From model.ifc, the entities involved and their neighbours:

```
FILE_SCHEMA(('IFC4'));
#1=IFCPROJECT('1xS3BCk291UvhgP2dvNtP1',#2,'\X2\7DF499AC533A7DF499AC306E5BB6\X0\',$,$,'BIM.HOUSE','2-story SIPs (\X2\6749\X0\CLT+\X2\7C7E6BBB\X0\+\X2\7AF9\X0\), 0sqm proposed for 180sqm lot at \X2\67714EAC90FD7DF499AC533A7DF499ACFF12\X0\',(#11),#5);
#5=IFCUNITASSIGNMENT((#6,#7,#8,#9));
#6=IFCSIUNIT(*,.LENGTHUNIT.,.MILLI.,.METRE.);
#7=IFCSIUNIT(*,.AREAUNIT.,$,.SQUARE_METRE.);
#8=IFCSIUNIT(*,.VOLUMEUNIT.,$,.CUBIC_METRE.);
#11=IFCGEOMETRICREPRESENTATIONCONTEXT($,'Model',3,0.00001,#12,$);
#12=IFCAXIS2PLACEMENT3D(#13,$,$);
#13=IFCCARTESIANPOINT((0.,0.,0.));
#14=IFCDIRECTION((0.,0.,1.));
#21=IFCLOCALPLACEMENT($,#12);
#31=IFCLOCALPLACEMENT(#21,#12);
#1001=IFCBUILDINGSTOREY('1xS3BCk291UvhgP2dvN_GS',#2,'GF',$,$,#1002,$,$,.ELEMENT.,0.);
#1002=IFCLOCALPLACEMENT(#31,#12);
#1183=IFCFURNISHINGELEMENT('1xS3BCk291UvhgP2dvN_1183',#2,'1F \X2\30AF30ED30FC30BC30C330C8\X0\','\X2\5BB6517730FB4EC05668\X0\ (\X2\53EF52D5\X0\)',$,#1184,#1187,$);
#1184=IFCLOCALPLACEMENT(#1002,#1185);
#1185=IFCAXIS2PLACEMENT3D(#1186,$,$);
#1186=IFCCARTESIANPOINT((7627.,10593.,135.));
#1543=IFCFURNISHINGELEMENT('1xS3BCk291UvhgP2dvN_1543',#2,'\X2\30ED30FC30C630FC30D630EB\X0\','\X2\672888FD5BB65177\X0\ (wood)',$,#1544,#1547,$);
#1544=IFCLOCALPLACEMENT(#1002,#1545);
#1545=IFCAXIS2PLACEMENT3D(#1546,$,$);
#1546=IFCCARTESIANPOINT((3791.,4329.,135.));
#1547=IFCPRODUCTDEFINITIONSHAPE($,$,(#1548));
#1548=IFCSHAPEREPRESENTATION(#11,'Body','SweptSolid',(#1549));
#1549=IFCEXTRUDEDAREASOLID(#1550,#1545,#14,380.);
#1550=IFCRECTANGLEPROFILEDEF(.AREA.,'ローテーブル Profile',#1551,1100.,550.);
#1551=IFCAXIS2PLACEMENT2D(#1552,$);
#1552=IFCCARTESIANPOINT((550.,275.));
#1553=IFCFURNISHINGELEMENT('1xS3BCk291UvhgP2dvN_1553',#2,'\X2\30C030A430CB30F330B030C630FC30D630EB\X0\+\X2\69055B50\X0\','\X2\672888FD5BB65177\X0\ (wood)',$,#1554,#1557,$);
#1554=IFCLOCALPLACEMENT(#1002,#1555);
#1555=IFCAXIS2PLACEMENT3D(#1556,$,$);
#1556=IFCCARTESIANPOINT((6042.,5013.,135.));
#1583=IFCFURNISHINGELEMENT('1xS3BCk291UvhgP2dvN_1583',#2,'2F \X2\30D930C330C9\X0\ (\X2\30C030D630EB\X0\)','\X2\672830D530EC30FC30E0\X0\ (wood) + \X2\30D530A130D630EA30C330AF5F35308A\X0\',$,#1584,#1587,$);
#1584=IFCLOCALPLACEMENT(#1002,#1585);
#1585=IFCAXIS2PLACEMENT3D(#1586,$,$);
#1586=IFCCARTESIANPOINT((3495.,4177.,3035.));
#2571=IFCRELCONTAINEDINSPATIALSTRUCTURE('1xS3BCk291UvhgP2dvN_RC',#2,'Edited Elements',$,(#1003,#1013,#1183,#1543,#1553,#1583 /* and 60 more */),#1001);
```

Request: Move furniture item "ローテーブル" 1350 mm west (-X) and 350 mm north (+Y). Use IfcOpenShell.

```python
import ifcopenshell
import ifcopenshell.api.geometry
import ifcopenshell.util.placement

model = ifcopenshell.open("model.ifc")

item = model.by_guid("1xS3BCk291UvhgP2dvN_1543")
matrix = ifcopenshell.util.placement.get_local_placement(item.ObjectPlacement)
matrix[0, 3] -= 1350.0
matrix[1, 3] += 350.0
ifcopenshell.api.geometry.edit_object_placement(model, product=item, matrix=matrix, is_si=False)

print(ifcopenshell.util.placement.get_local_placement(item.ObjectPlacement).round(3) + 0.0)

model.write("model_edited.ifc")
```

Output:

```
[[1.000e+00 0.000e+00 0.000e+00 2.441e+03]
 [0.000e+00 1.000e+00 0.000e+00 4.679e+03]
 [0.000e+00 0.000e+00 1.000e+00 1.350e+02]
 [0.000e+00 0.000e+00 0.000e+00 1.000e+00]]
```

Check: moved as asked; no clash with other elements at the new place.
